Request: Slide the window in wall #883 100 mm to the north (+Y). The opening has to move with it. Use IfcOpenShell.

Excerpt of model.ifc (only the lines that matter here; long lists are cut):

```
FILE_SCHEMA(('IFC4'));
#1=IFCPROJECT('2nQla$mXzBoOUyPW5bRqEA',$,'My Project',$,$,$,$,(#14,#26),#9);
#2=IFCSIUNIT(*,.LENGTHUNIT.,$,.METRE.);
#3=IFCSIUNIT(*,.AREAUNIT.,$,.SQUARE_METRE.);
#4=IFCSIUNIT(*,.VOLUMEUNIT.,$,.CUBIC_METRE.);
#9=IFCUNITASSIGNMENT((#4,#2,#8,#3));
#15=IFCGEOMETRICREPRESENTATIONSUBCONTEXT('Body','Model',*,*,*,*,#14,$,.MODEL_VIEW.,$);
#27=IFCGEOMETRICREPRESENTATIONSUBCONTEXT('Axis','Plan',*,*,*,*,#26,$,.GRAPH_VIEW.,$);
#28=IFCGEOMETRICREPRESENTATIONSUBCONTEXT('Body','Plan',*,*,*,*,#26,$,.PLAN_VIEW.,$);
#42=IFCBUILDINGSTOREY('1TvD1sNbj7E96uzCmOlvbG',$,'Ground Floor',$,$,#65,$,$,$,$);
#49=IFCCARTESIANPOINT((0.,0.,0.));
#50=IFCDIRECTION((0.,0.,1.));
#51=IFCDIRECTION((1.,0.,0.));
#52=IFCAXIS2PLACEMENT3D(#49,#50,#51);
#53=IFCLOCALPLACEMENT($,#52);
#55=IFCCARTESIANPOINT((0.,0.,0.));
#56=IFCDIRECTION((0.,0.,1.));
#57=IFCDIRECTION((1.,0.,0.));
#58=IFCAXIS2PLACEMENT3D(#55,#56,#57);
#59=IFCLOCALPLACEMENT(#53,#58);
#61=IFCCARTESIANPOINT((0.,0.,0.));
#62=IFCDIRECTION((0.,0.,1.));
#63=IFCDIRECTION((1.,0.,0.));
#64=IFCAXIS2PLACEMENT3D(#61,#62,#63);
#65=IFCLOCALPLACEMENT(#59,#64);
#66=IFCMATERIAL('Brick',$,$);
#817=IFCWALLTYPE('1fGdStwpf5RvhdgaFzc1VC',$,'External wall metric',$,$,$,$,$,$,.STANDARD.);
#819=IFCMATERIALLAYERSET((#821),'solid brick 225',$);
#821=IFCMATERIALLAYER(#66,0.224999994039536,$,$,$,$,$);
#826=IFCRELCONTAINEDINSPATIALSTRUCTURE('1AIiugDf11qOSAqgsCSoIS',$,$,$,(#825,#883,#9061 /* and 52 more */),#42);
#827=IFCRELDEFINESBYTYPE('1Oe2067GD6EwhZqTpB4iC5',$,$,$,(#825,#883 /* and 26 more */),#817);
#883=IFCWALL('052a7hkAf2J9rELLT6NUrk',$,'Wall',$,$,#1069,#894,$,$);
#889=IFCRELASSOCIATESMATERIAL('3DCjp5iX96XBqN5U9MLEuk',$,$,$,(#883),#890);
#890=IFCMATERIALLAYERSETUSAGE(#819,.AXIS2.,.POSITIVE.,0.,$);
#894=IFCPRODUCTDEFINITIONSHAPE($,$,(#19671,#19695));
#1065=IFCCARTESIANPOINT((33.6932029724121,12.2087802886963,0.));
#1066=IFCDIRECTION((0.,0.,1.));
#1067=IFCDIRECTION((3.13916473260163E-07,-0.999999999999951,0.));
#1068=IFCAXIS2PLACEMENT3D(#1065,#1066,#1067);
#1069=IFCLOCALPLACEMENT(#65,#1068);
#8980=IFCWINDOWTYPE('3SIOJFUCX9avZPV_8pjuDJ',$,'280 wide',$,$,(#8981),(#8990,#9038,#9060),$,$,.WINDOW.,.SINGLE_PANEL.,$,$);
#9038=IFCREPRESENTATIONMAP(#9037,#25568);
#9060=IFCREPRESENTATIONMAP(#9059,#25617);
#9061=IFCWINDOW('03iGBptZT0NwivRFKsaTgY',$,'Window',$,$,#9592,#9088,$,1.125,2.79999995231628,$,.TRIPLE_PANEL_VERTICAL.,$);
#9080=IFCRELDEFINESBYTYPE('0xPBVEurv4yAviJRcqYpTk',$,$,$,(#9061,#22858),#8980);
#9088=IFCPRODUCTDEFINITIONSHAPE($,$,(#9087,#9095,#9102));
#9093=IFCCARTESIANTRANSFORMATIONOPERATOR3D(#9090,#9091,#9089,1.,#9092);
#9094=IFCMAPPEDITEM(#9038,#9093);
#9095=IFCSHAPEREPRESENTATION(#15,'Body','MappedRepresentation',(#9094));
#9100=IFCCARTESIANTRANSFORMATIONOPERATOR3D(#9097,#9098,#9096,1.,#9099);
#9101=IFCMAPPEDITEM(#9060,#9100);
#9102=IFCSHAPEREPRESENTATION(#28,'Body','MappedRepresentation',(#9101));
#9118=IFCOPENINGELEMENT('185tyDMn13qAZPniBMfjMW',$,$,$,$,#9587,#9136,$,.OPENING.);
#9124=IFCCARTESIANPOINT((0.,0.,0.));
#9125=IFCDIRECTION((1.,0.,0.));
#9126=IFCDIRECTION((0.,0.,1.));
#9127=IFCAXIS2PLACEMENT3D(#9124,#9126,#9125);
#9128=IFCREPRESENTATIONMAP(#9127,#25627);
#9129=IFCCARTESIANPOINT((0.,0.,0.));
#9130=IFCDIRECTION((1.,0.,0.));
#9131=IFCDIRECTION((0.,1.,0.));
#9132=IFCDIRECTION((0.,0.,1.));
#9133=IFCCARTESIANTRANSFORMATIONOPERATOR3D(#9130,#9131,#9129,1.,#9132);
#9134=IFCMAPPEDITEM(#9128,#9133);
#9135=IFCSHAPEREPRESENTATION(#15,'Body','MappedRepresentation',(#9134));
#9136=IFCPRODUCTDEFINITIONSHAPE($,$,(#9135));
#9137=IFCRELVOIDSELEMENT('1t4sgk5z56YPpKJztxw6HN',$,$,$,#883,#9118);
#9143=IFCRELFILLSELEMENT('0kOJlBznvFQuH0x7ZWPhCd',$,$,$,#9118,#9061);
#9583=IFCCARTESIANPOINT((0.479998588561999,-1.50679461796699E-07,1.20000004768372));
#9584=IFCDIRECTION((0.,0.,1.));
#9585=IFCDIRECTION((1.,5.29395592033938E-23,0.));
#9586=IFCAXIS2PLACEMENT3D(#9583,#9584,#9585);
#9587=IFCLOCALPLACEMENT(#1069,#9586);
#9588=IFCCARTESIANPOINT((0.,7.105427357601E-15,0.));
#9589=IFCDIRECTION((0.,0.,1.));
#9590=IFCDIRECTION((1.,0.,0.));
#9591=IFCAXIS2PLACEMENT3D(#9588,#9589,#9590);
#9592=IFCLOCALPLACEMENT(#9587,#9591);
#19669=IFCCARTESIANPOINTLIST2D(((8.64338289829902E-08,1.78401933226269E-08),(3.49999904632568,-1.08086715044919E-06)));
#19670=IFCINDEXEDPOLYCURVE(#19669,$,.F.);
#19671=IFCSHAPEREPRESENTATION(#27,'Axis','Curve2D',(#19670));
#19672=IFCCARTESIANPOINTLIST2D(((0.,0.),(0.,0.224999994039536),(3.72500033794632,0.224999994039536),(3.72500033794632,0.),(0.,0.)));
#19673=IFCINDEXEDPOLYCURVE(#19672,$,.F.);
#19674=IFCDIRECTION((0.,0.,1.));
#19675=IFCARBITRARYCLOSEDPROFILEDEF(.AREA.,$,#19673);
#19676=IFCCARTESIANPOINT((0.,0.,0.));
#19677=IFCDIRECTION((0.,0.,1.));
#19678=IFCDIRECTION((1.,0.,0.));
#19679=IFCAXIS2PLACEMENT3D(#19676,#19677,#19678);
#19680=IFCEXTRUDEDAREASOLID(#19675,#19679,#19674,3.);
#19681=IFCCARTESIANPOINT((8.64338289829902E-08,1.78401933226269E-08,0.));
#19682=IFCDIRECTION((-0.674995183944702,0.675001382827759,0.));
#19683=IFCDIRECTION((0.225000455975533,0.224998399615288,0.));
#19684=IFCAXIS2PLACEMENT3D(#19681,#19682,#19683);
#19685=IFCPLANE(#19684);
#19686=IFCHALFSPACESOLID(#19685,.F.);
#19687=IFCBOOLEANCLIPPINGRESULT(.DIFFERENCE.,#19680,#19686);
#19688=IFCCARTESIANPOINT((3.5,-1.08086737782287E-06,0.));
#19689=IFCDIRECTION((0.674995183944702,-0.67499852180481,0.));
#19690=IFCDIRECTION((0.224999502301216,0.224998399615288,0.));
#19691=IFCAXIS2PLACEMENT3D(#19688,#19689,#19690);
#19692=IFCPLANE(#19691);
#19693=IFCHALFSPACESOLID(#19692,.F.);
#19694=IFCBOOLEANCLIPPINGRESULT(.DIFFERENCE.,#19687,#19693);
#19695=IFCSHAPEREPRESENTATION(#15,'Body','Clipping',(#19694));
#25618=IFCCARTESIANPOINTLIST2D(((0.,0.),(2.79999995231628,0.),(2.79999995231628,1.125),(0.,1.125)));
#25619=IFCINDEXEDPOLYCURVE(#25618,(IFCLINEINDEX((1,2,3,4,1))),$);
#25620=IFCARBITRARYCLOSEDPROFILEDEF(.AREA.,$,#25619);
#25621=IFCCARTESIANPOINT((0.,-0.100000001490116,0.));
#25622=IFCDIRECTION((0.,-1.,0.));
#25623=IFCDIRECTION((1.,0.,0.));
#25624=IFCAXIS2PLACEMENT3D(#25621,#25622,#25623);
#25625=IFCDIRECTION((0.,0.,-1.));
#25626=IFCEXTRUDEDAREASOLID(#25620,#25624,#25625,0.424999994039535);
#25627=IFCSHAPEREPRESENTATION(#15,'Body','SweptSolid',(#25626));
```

```python
import ifcopenshell
import ifcopenshell.api.geometry
import ifcopenshell.util.placement

model = ifcopenshell.open("model.ifc")

window = model.by_id(9061)
opening = window.FillsVoids[0].RelatingOpeningElement
wall = opening.VoidsElements[0].RelatingBuildingElement

wall_matrix = ifcopenshell.util.placement.get_local_placement(wall.ObjectPlacement)
shift = wall_matrix[:3, 0] * -0.1
before = ifcopenshell.util.placement.get_local_placement(window.ObjectPlacement)[:3, 3].copy()

# The window is placed relative to its opening, so it follows when the opening moves.
matrix = ifcopenshell.util.placement.get_local_placement(opening.ObjectPlacement)
matrix[:3, 3] += shift
ifcopenshell.api.geometry.edit_object_placement(
    model, product=opening, matrix=matrix, is_si=False, should_transform_children=True
)

after = ifcopenshell.util.placement.get_local_placement(window.ObjectPlacement)[:3, 3]
print("window moved by", (after - before).round(3) + 0.0)

model.write("model_updated.ifc")
```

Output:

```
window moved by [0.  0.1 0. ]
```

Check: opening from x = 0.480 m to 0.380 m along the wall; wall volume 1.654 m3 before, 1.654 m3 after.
